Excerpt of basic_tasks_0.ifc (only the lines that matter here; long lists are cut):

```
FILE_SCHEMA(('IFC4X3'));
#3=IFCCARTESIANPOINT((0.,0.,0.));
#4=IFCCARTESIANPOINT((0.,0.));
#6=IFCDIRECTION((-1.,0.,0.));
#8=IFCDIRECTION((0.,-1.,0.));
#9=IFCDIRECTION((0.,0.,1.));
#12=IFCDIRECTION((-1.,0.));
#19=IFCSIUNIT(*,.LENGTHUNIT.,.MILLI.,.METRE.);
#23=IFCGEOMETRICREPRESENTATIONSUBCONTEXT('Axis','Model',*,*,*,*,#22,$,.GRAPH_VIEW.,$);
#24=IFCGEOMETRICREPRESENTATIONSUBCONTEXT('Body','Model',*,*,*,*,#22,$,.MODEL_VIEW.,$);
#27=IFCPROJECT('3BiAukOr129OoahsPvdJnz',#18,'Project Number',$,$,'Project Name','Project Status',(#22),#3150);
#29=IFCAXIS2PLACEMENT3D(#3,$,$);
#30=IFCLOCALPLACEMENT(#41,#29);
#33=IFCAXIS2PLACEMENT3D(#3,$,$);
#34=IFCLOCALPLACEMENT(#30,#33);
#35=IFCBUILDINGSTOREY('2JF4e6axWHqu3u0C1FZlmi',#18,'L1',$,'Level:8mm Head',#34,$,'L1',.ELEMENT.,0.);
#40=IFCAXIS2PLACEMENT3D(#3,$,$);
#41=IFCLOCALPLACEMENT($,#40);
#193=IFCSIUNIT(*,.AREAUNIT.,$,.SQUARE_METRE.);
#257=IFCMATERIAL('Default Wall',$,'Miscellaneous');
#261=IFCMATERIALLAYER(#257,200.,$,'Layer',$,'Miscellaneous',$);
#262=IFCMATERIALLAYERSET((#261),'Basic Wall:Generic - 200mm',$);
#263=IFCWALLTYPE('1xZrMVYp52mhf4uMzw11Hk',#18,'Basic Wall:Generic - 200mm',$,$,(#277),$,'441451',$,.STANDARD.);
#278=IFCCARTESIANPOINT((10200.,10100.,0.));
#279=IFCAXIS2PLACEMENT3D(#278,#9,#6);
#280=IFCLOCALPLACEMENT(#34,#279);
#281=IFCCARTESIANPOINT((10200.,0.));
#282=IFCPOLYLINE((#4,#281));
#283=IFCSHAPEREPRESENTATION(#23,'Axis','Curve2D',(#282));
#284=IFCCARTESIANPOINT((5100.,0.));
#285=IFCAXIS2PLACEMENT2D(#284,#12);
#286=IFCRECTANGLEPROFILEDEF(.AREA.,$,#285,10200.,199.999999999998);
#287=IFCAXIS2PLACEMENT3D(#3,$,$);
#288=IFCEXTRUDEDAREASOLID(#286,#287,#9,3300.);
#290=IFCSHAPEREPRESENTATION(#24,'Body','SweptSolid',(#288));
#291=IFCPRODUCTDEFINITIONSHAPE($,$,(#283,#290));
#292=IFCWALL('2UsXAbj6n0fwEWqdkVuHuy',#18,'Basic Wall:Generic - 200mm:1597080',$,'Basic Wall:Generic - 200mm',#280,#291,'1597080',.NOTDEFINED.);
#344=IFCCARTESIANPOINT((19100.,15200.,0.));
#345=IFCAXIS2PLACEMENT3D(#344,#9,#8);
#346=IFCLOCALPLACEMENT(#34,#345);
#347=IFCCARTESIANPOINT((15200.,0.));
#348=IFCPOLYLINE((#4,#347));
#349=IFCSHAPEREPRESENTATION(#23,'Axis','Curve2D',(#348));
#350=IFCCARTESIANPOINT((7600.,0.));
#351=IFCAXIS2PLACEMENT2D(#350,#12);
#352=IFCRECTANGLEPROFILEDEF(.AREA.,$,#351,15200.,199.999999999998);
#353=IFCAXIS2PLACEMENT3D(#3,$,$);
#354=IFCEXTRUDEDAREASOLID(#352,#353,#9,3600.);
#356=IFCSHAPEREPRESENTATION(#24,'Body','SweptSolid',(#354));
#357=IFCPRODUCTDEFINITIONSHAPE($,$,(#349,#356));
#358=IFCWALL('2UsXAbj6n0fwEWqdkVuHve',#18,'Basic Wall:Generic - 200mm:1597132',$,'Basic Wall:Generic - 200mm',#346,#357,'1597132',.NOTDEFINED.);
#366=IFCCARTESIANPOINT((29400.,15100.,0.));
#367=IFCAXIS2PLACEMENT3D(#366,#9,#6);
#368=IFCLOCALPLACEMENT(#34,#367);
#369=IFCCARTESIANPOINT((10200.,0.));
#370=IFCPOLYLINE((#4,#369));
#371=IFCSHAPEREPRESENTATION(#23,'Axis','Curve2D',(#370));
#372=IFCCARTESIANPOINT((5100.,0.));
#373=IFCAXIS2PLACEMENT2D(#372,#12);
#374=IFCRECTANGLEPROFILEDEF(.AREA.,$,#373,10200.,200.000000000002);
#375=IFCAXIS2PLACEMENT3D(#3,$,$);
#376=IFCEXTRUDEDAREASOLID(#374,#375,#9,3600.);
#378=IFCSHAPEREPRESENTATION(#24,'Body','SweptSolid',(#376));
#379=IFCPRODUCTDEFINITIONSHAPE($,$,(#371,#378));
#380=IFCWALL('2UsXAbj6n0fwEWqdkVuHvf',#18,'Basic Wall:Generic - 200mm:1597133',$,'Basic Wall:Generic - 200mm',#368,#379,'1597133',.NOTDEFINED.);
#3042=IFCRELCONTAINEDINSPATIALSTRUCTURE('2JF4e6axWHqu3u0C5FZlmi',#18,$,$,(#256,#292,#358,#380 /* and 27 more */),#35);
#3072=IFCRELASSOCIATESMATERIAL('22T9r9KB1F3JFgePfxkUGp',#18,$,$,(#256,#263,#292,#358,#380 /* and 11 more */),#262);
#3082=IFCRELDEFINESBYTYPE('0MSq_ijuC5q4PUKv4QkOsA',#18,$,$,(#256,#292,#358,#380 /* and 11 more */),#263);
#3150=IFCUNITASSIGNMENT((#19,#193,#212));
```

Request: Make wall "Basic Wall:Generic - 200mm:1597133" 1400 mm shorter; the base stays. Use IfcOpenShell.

```python
import ifcopenshell
import ifcopenshell.geom
import ifcopenshell.util.representation
import ifcopenshell.util.shape
import ifcopenshell.util.unit

model = ifcopenshell.open("basic_tasks_0.ifc")
unit_scale = ifcopenshell.util.unit.calculate_unit_scale(model)
settings = ifcopenshell.geom.settings()


def volume(element):
    """Net volume in cubic metres, openings subtracted."""
    shape = ifcopenshell.geom.create_shape(settings, element)
    return ifcopenshell.util.shape.get_volume(shape.geometry)


wall = model.by_id(380)
before = volume(wall)

body = ifcopenshell.util.representation.get_representation(wall, "Model", "Body")
solid = body.Items[0]
old_height = solid.Depth
solid.Depth -= 1.4 / unit_scale
after = volume(wall)

print(f"height {old_height:g} -> {solid.Depth:g}, volume {before:.3f} -> {after:.3f} m3")

model.write("basic_tasks_0-out.ifc")
```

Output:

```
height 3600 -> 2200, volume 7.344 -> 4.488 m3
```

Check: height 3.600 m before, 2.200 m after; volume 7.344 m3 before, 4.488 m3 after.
